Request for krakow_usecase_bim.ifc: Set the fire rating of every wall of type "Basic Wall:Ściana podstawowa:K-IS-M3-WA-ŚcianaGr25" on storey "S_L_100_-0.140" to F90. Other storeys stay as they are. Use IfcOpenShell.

First a look at what the model holds.

```python
import ifcopenshell
import ifcopenshell.util.element

model = ifcopenshell.open("krakow_usecase_bim.ifc")
print(model.schema)
storey = next(s for s in model.by_type("IfcBuildingStorey") if s.Name == "S_L_100_-0.140")
walls = [e for e in ifcopenshell.util.element.get_decomposition(storey) if e.is_a("IfcWall")]
seen = {}
for e in walls:
    element_type = ifcopenshell.util.element.get_type(e)
    key = (element_type.Name if element_type != e and element_type else None, ifcopenshell.util.element.get_pset(e, "Pset_WallCommon", "FireRating"))
    seen[key] = seen.get(key, 0) + 1
for (name, value), count in sorted(seen.items(), key=str):
    print(count, "x", name, "|", value)
```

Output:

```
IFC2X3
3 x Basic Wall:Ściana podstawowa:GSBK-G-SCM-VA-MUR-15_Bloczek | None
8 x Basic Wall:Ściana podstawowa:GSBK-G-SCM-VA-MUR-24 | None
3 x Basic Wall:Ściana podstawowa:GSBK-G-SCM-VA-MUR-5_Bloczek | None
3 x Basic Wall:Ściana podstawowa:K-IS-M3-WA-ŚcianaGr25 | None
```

```python
import ifcopenshell
import ifcopenshell.api.pset
import ifcopenshell.util.element

model = ifcopenshell.open("krakow_usecase_bim.ifc")

storey = next(s for s in model.by_type("IfcBuildingStorey") if s.Name == "S_L_100_-0.140")
walls = [e for e in ifcopenshell.util.element.get_decomposition(storey) if e.is_a("IfcWall")]

count = 0
for e in walls:
    element_type = ifcopenshell.util.element.get_type(e)
    if element_type in (None, e) or element_type.Name != "Basic Wall:Ściana podstawowa:K-IS-M3-WA-ŚcianaGr25":
        continue
    # add_pset returns the element's existing set when there is one.
    pset = ifcopenshell.api.pset.add_pset(model, product=e, name="Pset_WallCommon")
    ifcopenshell.api.pset.edit_pset(model, pset=pset, properties={"FireRating": "F90"})
    count += 1

print(count, "walls updated")

model.write("krakow_usecase_bim_rev.ifc")
```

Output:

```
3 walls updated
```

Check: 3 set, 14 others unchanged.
